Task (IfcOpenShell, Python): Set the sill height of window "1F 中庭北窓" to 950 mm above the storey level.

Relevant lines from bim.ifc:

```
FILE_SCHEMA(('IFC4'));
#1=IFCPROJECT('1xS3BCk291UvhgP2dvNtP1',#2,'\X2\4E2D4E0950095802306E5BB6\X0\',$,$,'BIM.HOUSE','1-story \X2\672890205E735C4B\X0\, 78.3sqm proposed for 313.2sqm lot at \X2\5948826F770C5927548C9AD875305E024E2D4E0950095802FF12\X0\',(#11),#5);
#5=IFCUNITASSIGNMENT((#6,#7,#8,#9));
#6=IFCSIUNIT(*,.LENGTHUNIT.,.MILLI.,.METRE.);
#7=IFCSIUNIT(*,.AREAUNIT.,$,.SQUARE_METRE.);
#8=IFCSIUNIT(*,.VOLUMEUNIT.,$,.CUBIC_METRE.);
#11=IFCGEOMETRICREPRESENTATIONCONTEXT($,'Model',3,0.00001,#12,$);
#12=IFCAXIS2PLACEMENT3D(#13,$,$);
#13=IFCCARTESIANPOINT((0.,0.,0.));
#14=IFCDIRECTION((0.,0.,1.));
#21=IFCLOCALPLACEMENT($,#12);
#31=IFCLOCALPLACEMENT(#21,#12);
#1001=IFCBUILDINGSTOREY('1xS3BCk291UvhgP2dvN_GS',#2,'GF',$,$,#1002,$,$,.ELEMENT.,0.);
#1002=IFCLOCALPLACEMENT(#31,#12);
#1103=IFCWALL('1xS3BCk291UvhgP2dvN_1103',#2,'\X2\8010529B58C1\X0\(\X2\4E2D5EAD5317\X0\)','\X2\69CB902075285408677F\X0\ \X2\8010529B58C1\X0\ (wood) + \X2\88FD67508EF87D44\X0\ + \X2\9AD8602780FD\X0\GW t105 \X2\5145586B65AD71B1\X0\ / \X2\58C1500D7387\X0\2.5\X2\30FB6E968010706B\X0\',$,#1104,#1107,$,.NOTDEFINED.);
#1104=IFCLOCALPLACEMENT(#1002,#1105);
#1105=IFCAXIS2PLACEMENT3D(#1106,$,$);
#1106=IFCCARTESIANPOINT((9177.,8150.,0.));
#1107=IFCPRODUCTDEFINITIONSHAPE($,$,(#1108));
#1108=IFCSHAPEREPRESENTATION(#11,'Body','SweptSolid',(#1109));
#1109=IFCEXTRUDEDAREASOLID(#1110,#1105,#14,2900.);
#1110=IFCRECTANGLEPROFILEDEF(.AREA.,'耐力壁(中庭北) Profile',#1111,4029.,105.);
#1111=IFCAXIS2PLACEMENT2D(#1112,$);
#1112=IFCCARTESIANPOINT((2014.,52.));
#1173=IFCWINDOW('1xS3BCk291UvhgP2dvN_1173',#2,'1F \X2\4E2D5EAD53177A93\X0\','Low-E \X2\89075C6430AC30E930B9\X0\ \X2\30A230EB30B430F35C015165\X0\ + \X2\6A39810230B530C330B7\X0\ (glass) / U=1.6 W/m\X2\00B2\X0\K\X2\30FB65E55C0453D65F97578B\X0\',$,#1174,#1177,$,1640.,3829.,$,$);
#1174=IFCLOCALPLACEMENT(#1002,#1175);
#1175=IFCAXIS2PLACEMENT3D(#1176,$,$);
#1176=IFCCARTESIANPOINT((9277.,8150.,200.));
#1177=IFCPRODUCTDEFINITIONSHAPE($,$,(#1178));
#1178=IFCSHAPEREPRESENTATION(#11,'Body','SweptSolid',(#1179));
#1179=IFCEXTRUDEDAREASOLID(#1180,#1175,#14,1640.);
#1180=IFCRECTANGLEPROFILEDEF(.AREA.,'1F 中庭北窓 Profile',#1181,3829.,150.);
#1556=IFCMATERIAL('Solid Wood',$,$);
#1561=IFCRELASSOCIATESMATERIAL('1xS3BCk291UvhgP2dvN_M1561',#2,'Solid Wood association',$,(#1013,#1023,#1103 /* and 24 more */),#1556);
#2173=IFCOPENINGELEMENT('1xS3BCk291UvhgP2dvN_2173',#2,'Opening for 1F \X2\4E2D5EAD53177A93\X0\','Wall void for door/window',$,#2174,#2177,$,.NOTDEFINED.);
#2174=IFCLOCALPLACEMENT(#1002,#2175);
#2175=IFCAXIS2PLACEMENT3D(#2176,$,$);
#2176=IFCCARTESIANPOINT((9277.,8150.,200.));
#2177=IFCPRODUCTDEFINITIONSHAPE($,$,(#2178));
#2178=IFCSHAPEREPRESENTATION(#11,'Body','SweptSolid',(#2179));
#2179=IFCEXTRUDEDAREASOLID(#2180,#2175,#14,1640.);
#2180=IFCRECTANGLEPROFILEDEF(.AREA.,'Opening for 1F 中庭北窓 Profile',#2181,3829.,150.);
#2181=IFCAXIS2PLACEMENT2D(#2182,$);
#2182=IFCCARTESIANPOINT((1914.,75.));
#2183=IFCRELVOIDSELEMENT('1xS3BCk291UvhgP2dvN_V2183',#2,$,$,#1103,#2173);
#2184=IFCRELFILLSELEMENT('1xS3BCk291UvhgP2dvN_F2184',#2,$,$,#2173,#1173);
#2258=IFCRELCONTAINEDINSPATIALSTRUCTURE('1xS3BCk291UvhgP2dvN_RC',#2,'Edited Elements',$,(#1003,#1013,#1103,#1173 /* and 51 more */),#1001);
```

```python
import numpy as np
import ifcopenshell
import ifcopenshell.api.geometry
import ifcopenshell.geom
import ifcopenshell.util.element
import ifcopenshell.util.placement
import ifcopenshell.util.shape
import ifcopenshell.util.unit

model = ifcopenshell.open("bim.ifc")
unit_scale = ifcopenshell.util.unit.calculate_unit_scale(model)

window = model.by_guid("1xS3BCk291UvhgP2dvN_1173")
opening = window.FillsVoids[0].RelatingOpeningElement
storey = ifcopenshell.util.element.get_container(window, ifc_class="IfcBuildingStorey")
level = ifcopenshell.util.placement.get_local_placement(storey.ObjectPlacement)[2, 3]

# The opening's origin need not be at the sill, so measure its lowest point.
shape = ifcopenshell.geom.create_shape(ifcopenshell.geom.settings(), opening)
bottom = ifcopenshell.util.shape.get_shape_bottom_elevation(shape, shape.geometry) / unit_scale
dz = level + 950.0 - bottom

shift = np.array([0.0, 0.0, dz])
# The window is not placed relative to its opening, so move both.
for product in (opening, window):
    matrix = ifcopenshell.util.placement.get_local_placement(product.ObjectPlacement)
    matrix[:3, 3] += shift
    ifcopenshell.api.geometry.edit_object_placement(model, product=product, matrix=matrix, is_si=False)

print(f"moved by {dz * unit_scale:+.3f} m")

model.write("bim-out.ifc")
```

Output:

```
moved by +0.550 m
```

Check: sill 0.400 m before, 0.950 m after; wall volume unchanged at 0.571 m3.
